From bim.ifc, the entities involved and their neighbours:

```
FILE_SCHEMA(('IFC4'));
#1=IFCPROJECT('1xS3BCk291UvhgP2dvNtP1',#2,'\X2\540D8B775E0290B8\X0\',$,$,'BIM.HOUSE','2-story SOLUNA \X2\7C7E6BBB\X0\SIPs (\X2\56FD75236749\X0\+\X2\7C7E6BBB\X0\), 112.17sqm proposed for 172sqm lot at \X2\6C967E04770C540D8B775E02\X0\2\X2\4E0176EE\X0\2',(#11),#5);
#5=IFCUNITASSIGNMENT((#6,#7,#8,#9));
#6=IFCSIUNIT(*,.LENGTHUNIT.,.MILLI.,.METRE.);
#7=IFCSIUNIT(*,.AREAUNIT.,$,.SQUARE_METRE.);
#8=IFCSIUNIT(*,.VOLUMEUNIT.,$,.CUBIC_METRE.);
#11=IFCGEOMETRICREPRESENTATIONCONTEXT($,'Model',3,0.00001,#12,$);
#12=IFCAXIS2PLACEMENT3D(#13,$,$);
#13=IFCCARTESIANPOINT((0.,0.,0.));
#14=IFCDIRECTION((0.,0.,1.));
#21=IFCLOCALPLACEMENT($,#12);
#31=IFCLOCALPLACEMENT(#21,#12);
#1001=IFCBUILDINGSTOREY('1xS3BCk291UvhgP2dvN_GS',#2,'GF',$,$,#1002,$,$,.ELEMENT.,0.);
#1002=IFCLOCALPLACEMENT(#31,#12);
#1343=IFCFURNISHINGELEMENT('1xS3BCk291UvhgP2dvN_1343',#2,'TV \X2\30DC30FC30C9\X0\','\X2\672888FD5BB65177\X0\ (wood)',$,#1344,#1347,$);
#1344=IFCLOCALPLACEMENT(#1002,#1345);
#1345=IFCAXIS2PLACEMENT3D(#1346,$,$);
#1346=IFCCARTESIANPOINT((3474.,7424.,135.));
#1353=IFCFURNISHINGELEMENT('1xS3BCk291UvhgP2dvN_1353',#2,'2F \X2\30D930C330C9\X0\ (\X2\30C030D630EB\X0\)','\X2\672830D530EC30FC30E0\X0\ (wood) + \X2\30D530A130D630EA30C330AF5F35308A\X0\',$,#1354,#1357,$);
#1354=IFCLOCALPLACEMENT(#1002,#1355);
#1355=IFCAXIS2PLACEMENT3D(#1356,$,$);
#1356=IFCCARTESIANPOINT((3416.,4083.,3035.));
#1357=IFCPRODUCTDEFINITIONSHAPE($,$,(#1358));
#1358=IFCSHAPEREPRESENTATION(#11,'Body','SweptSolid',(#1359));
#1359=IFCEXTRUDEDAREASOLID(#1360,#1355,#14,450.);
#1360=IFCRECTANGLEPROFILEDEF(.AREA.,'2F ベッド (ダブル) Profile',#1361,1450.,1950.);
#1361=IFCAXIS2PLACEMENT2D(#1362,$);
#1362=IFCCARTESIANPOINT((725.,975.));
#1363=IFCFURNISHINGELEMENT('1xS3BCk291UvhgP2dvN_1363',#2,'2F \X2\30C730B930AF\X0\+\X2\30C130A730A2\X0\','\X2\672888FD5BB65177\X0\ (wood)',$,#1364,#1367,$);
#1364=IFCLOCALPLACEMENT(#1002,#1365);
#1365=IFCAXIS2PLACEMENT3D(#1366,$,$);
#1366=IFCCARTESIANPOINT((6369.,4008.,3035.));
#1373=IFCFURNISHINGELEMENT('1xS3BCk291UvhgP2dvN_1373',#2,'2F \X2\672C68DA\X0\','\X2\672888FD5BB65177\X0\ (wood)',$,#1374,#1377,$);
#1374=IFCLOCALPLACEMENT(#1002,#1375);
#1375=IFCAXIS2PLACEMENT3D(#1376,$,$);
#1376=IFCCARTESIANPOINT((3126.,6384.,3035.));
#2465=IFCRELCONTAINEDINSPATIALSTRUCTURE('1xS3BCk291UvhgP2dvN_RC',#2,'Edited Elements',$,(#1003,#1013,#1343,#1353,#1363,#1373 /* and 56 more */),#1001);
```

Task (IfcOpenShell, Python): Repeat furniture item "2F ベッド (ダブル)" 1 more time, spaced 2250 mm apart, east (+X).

```python
import numpy as np
import ifcopenshell
import ifcopenshell.api.geometry
import ifcopenshell.api.root
import ifcopenshell.util.element
import ifcopenshell.util.placement

model = ifcopenshell.open("bim.ifc")


def reuse_history(source, copy):
    """copy_class also copies each property set's owner history, people and application; keep the originals."""
    for rel in copy.IsDefinedBy:
        if rel.is_a("IfcRelDefinesByProperties") and (history := rel.RelatingPropertyDefinition.OwnerHistory):
            rel.RelatingPropertyDefinition.OwnerHistory = source.OwnerHistory
            ifcopenshell.util.element.remove_deep2(model, history)


source = model.by_guid("1xS3BCk291UvhgP2dvN_1353")
base = ifcopenshell.util.placement.get_local_placement(source.ObjectPlacement)
step = np.array([1.0, 0.0, 0.0]) * 2250.0

for i in range(1, 2):
    copy = ifcopenshell.api.root.copy_class(model, product=source)
    copy.Representation = ifcopenshell.util.element.copy_deep(
        model, source.Representation, exclude=["IfcGeometricRepresentationContext", "IfcRepresentationMap"]
    )
    reuse_history(source, copy)
    matrix = base.copy()
    matrix[:3, 3] += i * step
    print("added at", matrix[:3, 3].round(3) + 0.0)
    ifcopenshell.api.geometry.edit_object_placement(model, product=copy, matrix=matrix, is_si=False)

model.write("bim_updated.ifc")
```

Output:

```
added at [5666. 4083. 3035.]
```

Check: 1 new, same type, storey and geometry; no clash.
